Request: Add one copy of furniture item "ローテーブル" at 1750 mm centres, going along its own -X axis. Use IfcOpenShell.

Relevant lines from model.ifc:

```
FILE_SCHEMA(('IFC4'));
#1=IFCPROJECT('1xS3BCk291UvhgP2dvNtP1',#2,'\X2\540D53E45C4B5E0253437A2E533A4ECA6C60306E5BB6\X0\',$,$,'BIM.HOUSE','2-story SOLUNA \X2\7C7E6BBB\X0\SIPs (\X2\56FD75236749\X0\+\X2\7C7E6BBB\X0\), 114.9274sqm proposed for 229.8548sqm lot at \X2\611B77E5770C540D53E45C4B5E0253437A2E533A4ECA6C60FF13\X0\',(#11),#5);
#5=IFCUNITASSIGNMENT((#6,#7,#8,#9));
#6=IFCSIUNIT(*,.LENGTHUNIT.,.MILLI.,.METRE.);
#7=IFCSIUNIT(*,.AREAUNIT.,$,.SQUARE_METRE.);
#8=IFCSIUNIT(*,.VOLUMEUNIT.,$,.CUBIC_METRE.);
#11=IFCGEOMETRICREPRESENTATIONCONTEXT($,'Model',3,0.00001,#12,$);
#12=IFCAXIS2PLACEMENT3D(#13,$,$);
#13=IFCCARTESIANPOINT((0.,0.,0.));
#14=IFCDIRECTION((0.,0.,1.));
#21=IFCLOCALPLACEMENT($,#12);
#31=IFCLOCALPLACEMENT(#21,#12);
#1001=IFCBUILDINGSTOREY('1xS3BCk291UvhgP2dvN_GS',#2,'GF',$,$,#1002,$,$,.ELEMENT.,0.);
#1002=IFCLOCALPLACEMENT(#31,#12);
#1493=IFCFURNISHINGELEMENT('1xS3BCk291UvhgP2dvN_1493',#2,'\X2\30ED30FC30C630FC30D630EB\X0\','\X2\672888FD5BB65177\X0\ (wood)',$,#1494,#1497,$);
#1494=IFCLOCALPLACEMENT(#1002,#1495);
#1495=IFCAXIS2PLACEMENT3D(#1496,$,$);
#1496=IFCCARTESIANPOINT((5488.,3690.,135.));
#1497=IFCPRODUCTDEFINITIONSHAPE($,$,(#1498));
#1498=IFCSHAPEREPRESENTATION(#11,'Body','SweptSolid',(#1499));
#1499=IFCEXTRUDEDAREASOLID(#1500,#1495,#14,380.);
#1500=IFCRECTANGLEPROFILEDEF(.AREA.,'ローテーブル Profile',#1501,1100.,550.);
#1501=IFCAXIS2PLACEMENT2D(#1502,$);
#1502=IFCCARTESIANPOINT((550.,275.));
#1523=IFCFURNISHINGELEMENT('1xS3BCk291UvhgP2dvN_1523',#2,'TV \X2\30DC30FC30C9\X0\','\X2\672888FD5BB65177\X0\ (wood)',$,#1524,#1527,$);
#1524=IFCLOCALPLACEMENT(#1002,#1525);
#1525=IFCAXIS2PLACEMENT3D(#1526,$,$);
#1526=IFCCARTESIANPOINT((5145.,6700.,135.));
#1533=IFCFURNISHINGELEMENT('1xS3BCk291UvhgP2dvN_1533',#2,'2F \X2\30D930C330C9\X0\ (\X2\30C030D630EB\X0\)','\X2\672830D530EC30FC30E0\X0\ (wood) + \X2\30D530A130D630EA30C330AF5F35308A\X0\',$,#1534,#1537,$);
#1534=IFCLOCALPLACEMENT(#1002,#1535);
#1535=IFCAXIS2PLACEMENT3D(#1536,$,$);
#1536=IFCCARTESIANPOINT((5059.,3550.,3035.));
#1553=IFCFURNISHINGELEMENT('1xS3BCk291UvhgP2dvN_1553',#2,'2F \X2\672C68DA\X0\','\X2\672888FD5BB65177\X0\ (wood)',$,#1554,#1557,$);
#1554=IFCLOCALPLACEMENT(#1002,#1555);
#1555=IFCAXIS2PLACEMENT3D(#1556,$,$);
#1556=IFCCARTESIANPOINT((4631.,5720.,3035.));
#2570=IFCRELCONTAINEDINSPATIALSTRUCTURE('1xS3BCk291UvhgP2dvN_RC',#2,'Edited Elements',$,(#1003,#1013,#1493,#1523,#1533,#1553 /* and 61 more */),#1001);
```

```python
import ifcopenshell
import ifcopenshell.api.geometry
import ifcopenshell.api.root
import ifcopenshell.util.element
import ifcopenshell.util.placement
import ifcopenshell.util.unit

model = ifcopenshell.open("model.ifc")
unit_scale = ifcopenshell.util.unit.calculate_unit_scale(model)


def reuse_history(source, copy):
    """copy_class also copies each property set's owner history, people and application; keep the originals."""
    for rel in copy.IsDefinedBy:
        if rel.is_a("IfcRelDefinesByProperties") and (history := rel.RelatingPropertyDefinition.OwnerHistory):
            rel.RelatingPropertyDefinition.OwnerHistory = source.OwnerHistory
            ifcopenshell.util.element.remove_deep2(model, history)


source = model.by_guid("1xS3BCk291UvhgP2dvN_1493")
base = ifcopenshell.util.placement.get_local_placement(source.ObjectPlacement)
step = -base[:3, 0] * 1.75 / unit_scale

for i in range(1, 2):
    copy = ifcopenshell.api.root.copy_class(model, product=source)
    copy.Representation = ifcopenshell.util.element.copy_deep(
        model, source.Representation, exclude=["IfcGeometricRepresentationContext", "IfcRepresentationMap"]
    )
    reuse_history(source, copy)
    matrix = base.copy()
    matrix[:3, 3] += i * step
    print("added at", matrix[:3, 3].round(3) + 0.0)
    ifcopenshell.api.geometry.edit_object_placement(model, product=copy, matrix=matrix, is_si=False)

model.write("model_v2.ifc")
```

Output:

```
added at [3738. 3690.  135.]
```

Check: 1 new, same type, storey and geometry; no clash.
